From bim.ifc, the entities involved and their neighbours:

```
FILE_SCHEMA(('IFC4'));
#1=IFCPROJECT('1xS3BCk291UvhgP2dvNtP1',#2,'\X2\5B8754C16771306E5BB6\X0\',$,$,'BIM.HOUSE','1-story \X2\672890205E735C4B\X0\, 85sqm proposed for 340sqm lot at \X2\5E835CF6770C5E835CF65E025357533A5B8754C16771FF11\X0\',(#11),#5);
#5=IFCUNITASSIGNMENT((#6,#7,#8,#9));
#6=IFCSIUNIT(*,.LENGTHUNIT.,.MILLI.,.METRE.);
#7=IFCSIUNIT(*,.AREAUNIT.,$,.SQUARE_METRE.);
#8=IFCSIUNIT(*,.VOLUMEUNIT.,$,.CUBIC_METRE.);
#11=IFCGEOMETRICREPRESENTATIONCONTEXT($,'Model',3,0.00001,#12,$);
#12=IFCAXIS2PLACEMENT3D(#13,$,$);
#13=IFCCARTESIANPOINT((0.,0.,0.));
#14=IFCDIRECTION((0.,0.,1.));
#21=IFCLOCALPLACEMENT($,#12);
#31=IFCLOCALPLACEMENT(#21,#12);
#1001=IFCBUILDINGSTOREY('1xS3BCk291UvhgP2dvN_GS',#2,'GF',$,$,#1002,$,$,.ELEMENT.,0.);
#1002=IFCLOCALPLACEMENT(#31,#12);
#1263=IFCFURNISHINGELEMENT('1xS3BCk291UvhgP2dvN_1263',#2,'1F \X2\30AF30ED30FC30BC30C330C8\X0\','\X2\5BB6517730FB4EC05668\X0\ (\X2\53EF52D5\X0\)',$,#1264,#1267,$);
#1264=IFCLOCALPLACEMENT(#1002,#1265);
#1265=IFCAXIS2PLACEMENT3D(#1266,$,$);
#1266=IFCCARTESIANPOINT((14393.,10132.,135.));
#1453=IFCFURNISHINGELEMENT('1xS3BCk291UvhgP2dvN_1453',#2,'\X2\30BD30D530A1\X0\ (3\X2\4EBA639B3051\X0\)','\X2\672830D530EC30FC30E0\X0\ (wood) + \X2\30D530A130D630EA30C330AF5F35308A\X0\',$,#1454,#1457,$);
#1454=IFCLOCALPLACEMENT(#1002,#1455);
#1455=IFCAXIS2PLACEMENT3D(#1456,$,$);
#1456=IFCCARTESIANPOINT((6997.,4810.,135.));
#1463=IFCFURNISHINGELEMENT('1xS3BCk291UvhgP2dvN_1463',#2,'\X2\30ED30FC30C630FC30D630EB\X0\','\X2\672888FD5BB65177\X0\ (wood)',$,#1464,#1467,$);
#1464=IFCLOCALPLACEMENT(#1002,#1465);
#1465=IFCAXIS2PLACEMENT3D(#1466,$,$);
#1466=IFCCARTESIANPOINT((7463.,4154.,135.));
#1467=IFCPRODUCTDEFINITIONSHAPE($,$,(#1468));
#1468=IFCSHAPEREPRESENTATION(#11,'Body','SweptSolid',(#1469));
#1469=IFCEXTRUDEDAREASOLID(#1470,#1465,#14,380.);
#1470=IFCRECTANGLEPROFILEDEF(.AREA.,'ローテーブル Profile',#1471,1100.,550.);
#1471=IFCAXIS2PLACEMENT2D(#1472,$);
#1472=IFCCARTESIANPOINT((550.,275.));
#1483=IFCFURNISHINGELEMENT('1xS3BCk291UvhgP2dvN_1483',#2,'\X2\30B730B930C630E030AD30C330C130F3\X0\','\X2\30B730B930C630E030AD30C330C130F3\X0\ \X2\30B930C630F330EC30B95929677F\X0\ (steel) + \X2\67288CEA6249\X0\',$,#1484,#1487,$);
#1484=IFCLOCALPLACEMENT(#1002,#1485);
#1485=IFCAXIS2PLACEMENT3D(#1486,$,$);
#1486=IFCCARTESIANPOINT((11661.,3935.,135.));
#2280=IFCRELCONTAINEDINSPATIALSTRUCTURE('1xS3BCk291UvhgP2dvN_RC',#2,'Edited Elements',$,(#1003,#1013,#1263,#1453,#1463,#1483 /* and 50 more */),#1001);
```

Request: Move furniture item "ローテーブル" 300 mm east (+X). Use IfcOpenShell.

```python
import ifcopenshell
import ifcopenshell.api.geometry
import ifcopenshell.util.placement
import ifcopenshell.util.unit

model = ifcopenshell.open("bim.ifc")
unit_scale = ifcopenshell.util.unit.calculate_unit_scale(model)

item = model.by_guid("1xS3BCk291UvhgP2dvN_1463")
matrix = ifcopenshell.util.placement.get_local_placement(item.ObjectPlacement)
matrix[0, 3] += 0.3 / unit_scale
ifcopenshell.api.geometry.edit_object_placement(model, product=item, matrix=matrix, is_si=False)

print(ifcopenshell.util.placement.get_local_placement(item.ObjectPlacement).round(3) + 0.0)

model.write("bim_rev.ifc")
```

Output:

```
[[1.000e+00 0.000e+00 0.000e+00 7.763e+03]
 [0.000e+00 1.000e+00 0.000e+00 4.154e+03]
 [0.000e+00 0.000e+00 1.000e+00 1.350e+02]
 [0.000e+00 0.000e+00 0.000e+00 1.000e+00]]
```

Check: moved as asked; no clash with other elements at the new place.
